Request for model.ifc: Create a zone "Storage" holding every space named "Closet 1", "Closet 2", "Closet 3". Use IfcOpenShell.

First a look at what the model holds.

```python
import ifcopenshell

model = ifcopenshell.open("model.ifc")
print(model.schema)
seen = {}
for space in model.by_type("IfcSpace"):
    seen[space.LongName] = seen.get(space.LongName, 0) + 1
for name, count in sorted(seen.items(), key=str):
    print(count, "x", name)
print("zones:", [z.Name for z in model.by_type("IfcZone")][:20])
```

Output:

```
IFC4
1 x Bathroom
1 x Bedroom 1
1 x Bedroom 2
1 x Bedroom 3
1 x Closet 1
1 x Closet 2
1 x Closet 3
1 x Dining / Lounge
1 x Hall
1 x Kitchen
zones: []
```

```python
import ifcopenshell
import ifcopenshell.api.group
import ifcopenshell.api.root

model = ifcopenshell.open("model.ifc")

names = {"Closet 1", "Closet 2", "Closet 3"}
spaces = [s for s in model.by_type("IfcSpace") if s.LongName in names]

zone = ifcopenshell.api.root.create_entity(model, ifc_class="IfcZone", name="Storage")
ifcopenshell.api.group.assign_group(model, products=spaces, group=zone)
print(len(spaces), "spaces in", zone.Name)

model.write("model_updated.ifc")
```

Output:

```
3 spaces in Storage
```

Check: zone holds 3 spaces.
